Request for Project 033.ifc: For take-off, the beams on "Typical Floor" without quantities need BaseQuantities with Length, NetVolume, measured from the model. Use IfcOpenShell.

First a look at what the model holds.

```python
import ifcopenshell
import ifcopenshell.util.element
import ifcopenshell.util.unit

model = ifcopenshell.open("Project 033.ifc")
print(model.schema)
for unit_type in ("LENGTHUNIT", "AREAUNIT", "VOLUMEUNIT"):
    print(unit_type, ifcopenshell.util.unit.calculate_unit_scale(model, unit_type))
storey = next(s for s in model.by_type("IfcBuildingStorey") if s.Name == "Typical Floor")
beams = [e for e in ifcopenshell.util.element.get_decomposition(storey) if e.is_a("IfcBeam")]
for e in sorted(beams, key=lambda e: e.id()):
    print(e.id(), e.is_a(), e.Name, list(ifcopenshell.util.element.get_psets(e, qtos_only=True)), sep=" | ")
```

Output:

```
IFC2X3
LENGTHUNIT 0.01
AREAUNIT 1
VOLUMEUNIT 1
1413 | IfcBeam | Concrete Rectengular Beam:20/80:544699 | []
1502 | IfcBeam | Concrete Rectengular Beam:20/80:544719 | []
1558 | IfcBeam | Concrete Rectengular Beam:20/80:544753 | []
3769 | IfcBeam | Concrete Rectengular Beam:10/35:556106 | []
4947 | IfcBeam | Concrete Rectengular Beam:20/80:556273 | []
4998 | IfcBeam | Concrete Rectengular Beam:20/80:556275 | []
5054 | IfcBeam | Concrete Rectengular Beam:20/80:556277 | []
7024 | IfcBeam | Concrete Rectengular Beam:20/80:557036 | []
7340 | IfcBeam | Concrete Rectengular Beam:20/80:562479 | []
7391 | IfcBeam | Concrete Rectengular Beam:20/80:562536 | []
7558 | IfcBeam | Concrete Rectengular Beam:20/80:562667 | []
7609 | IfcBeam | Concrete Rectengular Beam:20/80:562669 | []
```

```python
import ifcopenshell
import ifcopenshell.api.pset
import ifcopenshell.geom
import ifcopenshell.util.element
import ifcopenshell.util.shape
import ifcopenshell.util.unit

model = ifcopenshell.open("Project 033.ifc")
unit_scale = ifcopenshell.util.unit.calculate_unit_scale(model)
volume_scale = ifcopenshell.util.unit.calculate_unit_scale(model, "VOLUMEUNIT")
settings = ifcopenshell.geom.settings()

storey = next(s for s in model.by_type("IfcBuildingStorey") if s.Name == "Typical Floor")
beams = [e for e in ifcopenshell.util.element.get_decomposition(storey) if e.is_a("IfcBeam")]

for e in sorted(beams, key=lambda e: e.id()):
    if ifcopenshell.util.element.get_psets(e, qtos_only=True, should_inherit=False):
        continue
    # Geometry comes back in metres, in the element's own axes.
    shape = ifcopenshell.geom.create_shape(settings, e)
    values = {
        "Length": ifcopenshell.util.shape.get_max_xyz(shape.geometry) / unit_scale,
        "NetVolume": ifcopenshell.util.shape.get_volume(shape.geometry) / volume_scale,
    }
    qto = ifcopenshell.api.pset.add_qto(model, product=e, name="BaseQuantities")
    ifcopenshell.api.pset.edit_qto(model, qto=qto, properties=values)
    print(e.id(), {k: round(v, 3) for k, v in values.items()})

model.write("Project 033-out.ifc")
```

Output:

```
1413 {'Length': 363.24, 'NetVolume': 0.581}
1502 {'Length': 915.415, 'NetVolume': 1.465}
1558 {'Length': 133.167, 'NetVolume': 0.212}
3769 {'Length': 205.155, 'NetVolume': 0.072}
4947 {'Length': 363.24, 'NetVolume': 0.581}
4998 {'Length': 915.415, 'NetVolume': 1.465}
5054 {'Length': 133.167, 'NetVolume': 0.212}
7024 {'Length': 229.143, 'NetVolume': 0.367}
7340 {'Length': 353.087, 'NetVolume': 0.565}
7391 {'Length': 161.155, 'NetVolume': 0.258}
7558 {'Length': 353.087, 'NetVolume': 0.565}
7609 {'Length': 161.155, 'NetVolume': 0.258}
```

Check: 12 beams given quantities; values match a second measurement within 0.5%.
